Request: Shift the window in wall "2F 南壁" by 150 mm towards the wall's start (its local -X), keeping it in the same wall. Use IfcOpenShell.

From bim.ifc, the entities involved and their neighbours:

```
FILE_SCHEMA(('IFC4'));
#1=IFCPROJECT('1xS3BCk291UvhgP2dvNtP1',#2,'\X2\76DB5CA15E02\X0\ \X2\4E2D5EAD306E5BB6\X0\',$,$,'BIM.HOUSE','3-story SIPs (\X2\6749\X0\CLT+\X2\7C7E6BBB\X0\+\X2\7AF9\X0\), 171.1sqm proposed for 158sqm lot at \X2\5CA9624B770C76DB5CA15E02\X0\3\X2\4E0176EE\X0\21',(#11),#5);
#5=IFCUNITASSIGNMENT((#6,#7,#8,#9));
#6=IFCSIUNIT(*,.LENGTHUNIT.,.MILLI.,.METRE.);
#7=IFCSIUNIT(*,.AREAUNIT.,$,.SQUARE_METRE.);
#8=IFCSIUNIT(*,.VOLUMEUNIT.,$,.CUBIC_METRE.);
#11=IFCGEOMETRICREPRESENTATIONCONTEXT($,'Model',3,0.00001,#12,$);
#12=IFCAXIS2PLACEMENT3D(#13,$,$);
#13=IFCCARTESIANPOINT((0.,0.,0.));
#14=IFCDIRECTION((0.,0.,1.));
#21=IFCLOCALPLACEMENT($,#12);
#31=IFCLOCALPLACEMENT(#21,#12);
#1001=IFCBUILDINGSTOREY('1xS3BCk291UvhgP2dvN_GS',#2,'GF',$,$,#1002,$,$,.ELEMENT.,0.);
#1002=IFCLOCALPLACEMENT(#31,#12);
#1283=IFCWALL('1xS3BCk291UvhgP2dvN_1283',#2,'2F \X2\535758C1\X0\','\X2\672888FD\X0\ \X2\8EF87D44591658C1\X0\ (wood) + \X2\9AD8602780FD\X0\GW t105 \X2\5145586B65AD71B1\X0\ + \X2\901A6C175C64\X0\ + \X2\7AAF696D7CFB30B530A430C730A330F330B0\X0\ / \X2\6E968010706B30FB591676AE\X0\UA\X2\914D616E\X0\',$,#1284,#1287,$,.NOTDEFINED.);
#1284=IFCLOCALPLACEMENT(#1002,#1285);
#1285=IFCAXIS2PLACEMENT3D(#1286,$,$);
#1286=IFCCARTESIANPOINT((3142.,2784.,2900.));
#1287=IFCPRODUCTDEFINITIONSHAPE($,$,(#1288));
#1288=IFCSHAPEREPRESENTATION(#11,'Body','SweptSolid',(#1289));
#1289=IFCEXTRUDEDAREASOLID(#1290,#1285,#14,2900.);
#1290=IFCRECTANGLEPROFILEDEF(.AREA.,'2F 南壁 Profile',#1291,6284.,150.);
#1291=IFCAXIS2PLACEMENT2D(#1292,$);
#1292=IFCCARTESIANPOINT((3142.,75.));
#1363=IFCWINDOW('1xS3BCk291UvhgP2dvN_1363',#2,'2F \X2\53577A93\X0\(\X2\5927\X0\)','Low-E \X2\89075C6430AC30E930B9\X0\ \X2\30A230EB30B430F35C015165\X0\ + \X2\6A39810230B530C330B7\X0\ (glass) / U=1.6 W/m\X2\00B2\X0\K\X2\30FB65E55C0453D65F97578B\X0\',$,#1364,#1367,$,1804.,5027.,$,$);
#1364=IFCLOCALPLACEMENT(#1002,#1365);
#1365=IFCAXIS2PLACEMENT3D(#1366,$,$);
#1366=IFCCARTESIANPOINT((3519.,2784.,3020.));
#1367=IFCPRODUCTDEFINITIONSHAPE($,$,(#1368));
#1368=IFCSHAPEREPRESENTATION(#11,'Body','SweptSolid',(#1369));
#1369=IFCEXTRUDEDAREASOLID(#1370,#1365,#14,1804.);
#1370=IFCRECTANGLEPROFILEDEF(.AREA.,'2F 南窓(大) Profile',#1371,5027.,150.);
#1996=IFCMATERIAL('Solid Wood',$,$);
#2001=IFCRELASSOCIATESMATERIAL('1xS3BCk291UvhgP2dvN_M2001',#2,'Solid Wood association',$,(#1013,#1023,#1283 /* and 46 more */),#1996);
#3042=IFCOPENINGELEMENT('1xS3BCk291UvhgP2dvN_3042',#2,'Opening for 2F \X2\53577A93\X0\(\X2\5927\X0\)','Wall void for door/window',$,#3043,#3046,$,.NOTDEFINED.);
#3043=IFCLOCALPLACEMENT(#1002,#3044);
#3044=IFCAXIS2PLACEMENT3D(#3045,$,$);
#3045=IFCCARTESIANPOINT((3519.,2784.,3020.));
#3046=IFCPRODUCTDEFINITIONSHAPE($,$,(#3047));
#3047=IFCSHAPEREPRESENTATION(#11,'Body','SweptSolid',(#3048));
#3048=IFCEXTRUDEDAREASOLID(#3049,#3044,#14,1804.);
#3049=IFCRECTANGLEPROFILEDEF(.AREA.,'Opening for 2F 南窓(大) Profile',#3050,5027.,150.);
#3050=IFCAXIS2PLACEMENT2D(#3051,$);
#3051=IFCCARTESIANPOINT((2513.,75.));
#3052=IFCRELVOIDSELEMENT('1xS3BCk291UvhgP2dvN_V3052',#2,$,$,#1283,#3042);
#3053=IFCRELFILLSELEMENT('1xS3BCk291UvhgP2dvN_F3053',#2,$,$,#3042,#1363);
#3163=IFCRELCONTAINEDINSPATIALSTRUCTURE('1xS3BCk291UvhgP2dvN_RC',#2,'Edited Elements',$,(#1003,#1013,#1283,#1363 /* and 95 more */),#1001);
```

```python
import ifcopenshell
import ifcopenshell.api.geometry
import ifcopenshell.util.placement

model = ifcopenshell.open("bim.ifc")

window = model.by_guid("1xS3BCk291UvhgP2dvN_1363")
opening = window.FillsVoids[0].RelatingOpeningElement
wall = opening.VoidsElements[0].RelatingBuildingElement

wall_matrix = ifcopenshell.util.placement.get_local_placement(wall.ObjectPlacement)
shift = wall_matrix[:3, 0] * -150.0
before = ifcopenshell.util.placement.get_local_placement(window.ObjectPlacement)[:3, 3].copy()

# The window is not placed relative to its opening, so move both.
for product in (opening, window):
    matrix = ifcopenshell.util.placement.get_local_placement(product.ObjectPlacement)
    matrix[:3, 3] += shift
    ifcopenshell.api.geometry.edit_object_placement(model, product=product, matrix=matrix, is_si=False)

after = ifcopenshell.util.placement.get_local_placement(window.ObjectPlacement)[:3, 3]
print("window moved by", (after - before).round(3) + 0.0)

model.write("bim_updated.ifc")
```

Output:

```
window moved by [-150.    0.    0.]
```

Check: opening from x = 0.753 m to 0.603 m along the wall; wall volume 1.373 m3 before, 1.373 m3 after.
